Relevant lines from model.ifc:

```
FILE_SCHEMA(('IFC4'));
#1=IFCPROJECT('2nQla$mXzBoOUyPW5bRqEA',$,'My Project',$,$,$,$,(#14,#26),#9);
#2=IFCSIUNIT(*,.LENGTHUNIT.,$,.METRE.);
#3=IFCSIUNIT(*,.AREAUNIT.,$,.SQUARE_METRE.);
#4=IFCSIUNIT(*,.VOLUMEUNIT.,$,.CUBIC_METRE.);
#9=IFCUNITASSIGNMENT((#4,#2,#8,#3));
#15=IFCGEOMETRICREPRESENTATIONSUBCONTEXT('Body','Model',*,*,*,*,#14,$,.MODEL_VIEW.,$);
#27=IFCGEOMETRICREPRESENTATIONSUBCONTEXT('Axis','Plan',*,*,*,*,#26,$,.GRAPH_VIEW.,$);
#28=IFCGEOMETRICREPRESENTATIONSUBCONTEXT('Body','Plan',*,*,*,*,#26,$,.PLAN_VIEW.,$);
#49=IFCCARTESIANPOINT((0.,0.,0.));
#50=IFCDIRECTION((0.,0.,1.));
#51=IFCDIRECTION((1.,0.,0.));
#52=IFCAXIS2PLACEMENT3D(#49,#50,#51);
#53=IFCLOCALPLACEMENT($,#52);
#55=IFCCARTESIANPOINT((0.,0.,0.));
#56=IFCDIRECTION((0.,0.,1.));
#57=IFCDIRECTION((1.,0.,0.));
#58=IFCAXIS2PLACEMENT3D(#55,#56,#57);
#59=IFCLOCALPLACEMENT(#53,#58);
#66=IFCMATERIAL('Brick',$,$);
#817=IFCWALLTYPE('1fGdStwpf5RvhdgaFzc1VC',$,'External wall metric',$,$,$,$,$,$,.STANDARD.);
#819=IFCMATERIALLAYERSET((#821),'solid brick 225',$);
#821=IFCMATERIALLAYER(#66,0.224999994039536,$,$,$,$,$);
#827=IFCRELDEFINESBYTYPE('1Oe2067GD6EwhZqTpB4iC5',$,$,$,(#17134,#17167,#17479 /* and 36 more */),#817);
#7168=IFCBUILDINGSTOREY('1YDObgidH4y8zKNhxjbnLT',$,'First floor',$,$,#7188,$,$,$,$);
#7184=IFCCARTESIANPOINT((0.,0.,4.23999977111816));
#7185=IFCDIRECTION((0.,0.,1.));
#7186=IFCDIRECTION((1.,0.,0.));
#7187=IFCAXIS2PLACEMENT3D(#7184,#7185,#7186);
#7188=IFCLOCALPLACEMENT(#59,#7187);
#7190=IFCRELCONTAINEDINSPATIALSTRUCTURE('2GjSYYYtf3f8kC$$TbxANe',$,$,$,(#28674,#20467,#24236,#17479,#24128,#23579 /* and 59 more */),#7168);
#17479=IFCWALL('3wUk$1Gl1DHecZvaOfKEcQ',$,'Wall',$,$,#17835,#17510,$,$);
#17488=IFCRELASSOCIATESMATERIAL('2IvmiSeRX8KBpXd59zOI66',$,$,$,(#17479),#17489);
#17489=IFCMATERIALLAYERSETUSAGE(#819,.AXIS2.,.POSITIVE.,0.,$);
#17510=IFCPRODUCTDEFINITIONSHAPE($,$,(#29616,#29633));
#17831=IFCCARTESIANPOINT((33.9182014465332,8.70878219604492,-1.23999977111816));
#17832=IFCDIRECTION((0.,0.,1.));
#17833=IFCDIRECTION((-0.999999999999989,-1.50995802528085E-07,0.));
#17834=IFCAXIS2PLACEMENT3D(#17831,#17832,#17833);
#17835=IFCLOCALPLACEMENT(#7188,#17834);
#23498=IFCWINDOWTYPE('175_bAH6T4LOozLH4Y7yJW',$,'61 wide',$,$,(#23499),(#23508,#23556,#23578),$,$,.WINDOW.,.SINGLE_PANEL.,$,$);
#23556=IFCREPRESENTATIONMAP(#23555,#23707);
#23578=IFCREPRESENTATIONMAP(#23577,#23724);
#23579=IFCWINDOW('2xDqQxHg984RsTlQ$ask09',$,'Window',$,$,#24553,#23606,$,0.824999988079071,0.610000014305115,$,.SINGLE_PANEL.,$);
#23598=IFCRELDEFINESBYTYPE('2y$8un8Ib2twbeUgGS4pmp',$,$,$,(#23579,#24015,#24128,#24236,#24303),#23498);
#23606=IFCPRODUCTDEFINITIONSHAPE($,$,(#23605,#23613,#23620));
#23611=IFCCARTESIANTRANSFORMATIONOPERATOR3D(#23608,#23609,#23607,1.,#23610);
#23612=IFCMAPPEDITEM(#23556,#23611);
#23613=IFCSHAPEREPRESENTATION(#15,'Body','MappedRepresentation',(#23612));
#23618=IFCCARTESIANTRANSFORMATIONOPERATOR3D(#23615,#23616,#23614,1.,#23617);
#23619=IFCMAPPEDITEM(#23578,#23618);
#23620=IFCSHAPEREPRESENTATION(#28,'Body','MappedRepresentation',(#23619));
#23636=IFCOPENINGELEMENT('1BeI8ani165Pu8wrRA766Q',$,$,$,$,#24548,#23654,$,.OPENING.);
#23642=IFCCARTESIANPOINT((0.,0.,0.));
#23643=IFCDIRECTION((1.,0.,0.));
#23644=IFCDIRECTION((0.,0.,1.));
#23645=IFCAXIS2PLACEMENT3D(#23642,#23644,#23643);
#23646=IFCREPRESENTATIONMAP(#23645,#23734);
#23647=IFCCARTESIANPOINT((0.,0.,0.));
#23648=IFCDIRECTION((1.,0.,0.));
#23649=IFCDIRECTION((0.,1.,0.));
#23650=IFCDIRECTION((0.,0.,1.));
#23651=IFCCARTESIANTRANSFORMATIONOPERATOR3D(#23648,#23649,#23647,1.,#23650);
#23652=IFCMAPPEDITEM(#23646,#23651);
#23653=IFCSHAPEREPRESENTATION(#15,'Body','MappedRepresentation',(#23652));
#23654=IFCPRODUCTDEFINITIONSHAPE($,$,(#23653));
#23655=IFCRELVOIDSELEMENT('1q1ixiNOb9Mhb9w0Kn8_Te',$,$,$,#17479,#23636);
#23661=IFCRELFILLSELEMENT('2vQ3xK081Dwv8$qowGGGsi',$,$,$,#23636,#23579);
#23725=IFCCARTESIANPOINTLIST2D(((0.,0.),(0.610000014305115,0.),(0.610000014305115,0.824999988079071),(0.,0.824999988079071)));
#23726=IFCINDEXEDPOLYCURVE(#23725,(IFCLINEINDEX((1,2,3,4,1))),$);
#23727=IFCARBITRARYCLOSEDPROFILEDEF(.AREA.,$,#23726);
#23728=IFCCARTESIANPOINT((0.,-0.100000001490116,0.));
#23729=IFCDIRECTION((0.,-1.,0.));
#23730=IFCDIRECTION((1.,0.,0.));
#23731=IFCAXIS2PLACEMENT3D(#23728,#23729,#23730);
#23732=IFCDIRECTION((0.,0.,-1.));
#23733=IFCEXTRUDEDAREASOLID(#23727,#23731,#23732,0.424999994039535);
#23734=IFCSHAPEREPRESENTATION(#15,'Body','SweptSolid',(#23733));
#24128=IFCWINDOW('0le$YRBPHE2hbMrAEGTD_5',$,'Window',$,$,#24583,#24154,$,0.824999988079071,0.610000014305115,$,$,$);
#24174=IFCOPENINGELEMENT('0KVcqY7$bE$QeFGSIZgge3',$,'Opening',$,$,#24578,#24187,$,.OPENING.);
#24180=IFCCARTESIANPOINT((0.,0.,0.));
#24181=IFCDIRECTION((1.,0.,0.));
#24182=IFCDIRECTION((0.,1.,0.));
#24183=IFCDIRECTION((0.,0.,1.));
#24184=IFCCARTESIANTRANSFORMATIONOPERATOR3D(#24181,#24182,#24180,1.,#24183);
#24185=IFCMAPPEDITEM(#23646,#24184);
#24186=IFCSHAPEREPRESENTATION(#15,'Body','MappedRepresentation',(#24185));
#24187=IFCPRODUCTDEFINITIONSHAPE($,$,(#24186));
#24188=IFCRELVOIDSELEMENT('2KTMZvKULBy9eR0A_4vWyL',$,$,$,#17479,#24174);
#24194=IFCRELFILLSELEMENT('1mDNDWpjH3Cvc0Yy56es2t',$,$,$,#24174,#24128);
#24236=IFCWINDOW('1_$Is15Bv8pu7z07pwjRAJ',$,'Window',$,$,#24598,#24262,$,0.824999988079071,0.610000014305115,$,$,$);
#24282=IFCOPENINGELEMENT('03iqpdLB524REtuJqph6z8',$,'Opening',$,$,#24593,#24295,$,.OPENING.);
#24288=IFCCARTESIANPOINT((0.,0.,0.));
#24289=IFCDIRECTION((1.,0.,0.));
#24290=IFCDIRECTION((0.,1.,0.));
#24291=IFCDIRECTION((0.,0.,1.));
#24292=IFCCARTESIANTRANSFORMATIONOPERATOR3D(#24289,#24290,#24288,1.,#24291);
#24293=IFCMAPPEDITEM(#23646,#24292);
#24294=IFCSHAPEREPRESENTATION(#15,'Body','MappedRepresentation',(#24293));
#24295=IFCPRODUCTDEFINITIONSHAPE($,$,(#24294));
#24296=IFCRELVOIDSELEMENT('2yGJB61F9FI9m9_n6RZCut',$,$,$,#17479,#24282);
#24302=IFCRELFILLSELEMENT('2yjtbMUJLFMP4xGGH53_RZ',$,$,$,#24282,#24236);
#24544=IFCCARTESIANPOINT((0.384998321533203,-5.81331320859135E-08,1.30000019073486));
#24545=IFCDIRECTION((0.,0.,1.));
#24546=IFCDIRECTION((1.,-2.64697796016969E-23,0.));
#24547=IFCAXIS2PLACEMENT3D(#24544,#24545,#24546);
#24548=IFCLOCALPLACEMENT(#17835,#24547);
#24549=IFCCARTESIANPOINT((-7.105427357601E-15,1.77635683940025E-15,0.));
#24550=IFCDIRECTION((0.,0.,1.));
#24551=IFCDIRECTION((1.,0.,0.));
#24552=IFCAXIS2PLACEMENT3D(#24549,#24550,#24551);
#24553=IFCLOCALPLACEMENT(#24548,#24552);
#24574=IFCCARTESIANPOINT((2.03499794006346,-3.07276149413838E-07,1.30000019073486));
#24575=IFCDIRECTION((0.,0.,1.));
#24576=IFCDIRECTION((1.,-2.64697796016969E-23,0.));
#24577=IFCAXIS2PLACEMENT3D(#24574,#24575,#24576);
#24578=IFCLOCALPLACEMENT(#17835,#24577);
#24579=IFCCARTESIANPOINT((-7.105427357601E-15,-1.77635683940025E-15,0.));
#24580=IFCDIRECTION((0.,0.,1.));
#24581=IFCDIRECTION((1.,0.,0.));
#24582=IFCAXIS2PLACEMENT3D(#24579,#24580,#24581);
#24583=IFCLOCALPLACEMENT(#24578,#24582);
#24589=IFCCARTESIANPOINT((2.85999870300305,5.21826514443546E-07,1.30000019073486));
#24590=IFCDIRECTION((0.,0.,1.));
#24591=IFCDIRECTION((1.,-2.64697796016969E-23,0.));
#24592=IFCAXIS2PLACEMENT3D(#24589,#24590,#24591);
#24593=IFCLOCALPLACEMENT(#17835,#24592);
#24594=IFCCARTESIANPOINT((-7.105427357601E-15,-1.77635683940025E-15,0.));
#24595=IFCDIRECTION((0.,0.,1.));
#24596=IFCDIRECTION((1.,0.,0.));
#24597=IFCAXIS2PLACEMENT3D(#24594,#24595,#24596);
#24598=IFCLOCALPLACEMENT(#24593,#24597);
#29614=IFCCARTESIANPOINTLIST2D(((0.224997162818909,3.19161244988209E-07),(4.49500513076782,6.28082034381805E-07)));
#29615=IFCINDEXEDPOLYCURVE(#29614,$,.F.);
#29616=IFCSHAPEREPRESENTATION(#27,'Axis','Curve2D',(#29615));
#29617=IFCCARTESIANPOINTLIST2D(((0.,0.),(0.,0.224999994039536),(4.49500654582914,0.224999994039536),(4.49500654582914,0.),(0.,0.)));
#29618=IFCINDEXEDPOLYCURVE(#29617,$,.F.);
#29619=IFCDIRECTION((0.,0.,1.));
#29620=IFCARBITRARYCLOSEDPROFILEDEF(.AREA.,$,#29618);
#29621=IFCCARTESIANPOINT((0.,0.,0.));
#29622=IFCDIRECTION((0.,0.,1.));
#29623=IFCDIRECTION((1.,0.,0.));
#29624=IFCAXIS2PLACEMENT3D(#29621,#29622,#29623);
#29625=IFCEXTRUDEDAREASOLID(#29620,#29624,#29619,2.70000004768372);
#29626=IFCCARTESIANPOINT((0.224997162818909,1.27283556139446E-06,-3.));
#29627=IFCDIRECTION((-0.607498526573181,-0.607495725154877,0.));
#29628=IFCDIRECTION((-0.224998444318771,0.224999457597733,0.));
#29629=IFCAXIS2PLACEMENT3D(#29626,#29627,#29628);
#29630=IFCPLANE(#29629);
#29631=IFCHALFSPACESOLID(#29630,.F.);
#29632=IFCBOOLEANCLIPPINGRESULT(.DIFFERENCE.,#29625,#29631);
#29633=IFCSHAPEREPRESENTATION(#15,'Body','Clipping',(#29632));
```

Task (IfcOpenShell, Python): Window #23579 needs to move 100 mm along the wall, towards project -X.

```python
import ifcopenshell
import ifcopenshell.api.geometry
import ifcopenshell.util.placement
import ifcopenshell.util.unit

model = ifcopenshell.open("model.ifc")
unit_scale = ifcopenshell.util.unit.calculate_unit_scale(model)

window = model.by_guid("2xDqQxHg984RsTlQ$ask09")
opening = window.FillsVoids[0].RelatingOpeningElement
wall = opening.VoidsElements[0].RelatingBuildingElement

wall_matrix = ifcopenshell.util.placement.get_local_placement(wall.ObjectPlacement)
shift = wall_matrix[:3, 0] * 0.1 / unit_scale
before = ifcopenshell.util.placement.get_local_placement(window.ObjectPlacement)[:3, 3].copy()

# The window is placed relative to its opening, so it follows when the opening moves.
matrix = ifcopenshell.util.placement.get_local_placement(opening.ObjectPlacement)
matrix[:3, 3] += shift
ifcopenshell.api.geometry.edit_object_placement(
    model, product=opening, matrix=matrix, is_si=False, should_transform_children=True
)

after = ifcopenshell.util.placement.get_local_placement(window.ObjectPlacement)[:3, 3]
print("window moved by", (after - before).round(3) + 0.0)

model.write("model_edited.ifc")
```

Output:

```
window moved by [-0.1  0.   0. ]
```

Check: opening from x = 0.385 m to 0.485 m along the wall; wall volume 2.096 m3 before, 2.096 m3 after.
